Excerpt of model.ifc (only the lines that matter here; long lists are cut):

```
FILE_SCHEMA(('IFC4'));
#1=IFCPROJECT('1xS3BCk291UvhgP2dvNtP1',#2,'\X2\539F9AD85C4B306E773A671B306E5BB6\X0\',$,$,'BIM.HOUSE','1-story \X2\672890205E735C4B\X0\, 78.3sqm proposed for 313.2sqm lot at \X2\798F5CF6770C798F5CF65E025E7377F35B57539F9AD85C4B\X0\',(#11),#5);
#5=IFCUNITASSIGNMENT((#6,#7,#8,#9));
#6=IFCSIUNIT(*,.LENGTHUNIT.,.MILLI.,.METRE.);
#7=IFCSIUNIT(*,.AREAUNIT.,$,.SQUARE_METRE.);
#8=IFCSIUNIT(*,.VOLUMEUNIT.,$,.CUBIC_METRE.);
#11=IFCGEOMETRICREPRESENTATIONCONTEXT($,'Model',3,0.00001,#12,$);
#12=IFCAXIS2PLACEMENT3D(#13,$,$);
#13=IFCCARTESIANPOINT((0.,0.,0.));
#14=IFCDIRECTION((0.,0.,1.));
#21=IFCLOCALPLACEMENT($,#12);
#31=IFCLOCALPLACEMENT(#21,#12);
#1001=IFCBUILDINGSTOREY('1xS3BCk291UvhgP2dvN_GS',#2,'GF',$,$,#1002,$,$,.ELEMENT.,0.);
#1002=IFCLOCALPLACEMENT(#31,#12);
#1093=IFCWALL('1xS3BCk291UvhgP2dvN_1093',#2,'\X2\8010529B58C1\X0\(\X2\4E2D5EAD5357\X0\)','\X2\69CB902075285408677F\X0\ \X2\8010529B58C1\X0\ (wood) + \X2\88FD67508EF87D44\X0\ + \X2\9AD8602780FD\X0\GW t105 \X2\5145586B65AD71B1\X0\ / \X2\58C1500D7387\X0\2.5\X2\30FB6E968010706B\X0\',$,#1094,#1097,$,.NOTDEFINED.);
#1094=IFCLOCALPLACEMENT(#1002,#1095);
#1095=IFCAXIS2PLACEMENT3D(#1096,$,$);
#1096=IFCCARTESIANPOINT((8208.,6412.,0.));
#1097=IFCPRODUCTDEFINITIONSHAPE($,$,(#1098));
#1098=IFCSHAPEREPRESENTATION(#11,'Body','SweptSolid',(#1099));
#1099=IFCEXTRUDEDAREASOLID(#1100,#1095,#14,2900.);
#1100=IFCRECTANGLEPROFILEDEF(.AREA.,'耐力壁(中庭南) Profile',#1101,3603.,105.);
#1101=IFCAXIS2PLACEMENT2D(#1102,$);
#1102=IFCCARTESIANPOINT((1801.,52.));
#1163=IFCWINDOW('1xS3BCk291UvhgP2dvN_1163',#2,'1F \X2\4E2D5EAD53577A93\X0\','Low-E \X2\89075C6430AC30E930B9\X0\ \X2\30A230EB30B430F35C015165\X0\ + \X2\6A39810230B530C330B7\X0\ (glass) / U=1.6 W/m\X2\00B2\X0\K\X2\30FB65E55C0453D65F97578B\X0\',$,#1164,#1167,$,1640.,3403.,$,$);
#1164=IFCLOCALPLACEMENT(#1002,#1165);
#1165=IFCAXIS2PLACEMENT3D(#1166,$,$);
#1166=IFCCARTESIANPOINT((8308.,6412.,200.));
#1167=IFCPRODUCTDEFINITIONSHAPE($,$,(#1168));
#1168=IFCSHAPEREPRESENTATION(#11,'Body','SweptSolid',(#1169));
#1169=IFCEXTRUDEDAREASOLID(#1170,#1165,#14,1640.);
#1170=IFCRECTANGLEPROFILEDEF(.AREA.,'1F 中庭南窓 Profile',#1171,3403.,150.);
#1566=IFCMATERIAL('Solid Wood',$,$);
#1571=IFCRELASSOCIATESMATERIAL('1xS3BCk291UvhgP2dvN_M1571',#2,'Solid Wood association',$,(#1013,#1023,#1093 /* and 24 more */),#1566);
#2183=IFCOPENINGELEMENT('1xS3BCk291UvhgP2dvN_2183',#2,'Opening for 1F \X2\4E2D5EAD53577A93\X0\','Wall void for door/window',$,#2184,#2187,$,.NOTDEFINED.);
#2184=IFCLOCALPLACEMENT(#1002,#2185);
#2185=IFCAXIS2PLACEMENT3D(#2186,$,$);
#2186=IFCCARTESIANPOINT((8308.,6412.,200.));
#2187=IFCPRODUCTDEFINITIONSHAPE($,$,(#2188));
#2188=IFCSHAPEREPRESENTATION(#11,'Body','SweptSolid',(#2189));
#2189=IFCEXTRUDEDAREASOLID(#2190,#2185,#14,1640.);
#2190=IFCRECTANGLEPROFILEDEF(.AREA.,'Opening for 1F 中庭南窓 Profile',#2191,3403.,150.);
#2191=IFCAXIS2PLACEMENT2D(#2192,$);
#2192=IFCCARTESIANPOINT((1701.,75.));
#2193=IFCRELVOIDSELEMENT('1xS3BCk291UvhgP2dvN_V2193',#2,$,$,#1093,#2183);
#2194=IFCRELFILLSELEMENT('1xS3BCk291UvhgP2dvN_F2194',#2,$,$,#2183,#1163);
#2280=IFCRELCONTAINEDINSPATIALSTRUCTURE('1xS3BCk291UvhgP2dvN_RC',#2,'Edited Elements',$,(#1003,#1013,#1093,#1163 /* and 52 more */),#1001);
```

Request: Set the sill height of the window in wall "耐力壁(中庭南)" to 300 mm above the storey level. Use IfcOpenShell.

```python
import numpy as np
import ifcopenshell
import ifcopenshell.api.geometry
import ifcopenshell.geom
import ifcopenshell.util.element
import ifcopenshell.util.placement
import ifcopenshell.util.shape
import ifcopenshell.util.unit

model = ifcopenshell.open("model.ifc")
unit_scale = ifcopenshell.util.unit.calculate_unit_scale(model)

window = model.by_guid("1xS3BCk291UvhgP2dvN_1163")
opening = window.FillsVoids[0].RelatingOpeningElement
storey = ifcopenshell.util.element.get_container(window, ifc_class="IfcBuildingStorey")
level = ifcopenshell.util.placement.get_local_placement(storey.ObjectPlacement)[2, 3]

# The opening's origin need not be at the sill, so measure its lowest point.
shape = ifcopenshell.geom.create_shape(ifcopenshell.geom.settings(), opening)
bottom = ifcopenshell.util.shape.get_shape_bottom_elevation(shape, shape.geometry) / unit_scale
dz = level + 300.0 - bottom

shift = np.array([0.0, 0.0, dz])
# The window is not placed relative to its opening, so move both.
for product in (opening, window):
    matrix = ifcopenshell.util.placement.get_local_placement(product.ObjectPlacement)
    matrix[:3, 3] += shift
    ifcopenshell.api.geometry.edit_object_placement(model, product=product, matrix=matrix, is_si=False)

print(f"moved by {dz * unit_scale:+.3f} m")

model.write("model_v2.ifc")
```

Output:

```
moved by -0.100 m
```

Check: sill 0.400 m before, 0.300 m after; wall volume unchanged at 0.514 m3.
